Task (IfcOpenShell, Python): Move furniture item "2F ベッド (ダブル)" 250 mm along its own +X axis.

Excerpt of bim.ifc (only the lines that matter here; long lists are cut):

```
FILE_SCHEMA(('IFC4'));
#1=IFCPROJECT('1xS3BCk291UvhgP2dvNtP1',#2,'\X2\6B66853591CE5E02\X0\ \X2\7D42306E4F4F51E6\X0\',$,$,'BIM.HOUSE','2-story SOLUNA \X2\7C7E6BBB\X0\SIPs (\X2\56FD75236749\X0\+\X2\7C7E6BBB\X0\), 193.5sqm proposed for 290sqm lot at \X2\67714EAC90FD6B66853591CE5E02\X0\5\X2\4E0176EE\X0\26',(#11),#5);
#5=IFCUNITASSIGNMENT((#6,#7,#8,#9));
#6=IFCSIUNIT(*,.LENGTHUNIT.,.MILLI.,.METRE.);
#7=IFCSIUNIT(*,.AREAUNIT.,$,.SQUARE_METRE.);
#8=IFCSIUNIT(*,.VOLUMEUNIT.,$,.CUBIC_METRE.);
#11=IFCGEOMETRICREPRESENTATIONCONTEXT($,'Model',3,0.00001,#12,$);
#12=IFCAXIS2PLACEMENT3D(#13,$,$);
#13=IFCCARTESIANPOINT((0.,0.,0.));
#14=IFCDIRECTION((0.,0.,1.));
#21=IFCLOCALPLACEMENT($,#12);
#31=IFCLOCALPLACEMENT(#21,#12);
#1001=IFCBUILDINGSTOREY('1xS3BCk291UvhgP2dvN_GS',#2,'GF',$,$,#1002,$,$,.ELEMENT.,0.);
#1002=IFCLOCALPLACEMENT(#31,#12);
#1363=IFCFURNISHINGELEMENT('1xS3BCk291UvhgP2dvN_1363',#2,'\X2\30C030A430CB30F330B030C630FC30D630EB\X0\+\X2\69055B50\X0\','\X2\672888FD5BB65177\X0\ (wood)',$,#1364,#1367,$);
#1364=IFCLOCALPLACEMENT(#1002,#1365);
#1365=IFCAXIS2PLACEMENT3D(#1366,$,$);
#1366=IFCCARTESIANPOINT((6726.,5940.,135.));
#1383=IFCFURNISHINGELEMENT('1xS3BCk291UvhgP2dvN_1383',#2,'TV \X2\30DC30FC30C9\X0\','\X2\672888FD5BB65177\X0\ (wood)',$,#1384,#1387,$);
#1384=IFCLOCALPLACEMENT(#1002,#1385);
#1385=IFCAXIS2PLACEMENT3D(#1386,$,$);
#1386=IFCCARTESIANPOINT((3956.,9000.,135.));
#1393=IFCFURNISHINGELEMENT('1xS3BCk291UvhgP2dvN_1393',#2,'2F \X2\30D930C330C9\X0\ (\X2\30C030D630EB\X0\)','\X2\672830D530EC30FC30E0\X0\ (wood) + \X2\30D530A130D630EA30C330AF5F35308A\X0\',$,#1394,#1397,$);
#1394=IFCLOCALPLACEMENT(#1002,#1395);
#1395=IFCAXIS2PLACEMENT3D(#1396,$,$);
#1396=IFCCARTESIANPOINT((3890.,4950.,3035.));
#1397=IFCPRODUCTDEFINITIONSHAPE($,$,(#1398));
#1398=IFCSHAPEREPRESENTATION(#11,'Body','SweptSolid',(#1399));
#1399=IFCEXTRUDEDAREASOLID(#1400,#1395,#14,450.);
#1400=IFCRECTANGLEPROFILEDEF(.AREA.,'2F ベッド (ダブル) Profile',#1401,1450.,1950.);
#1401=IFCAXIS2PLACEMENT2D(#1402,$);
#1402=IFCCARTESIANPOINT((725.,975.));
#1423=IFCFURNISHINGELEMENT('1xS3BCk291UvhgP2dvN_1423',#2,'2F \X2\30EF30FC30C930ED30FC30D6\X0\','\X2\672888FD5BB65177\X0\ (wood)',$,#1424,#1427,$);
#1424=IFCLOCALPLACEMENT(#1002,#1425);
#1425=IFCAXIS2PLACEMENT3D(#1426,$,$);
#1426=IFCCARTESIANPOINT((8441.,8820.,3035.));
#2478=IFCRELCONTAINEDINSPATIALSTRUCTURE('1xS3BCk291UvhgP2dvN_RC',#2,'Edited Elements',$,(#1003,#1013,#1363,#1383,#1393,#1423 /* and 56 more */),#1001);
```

```python
import ifcopenshell
import ifcopenshell.api.geometry
import ifcopenshell.util.placement
import ifcopenshell.util.unit

model = ifcopenshell.open("bim.ifc")
unit_scale = ifcopenshell.util.unit.calculate_unit_scale(model)

item = model.by_guid("1xS3BCk291UvhgP2dvN_1393")
matrix = ifcopenshell.util.placement.get_local_placement(item.ObjectPlacement)
matrix[:3, 3] += matrix[:3, 0] * 0.25 / unit_scale
ifcopenshell.api.geometry.edit_object_placement(model, product=item, matrix=matrix, is_si=False)

print(ifcopenshell.util.placement.get_local_placement(item.ObjectPlacement).round(3) + 0.0)

model.write("bim_edited.ifc")
```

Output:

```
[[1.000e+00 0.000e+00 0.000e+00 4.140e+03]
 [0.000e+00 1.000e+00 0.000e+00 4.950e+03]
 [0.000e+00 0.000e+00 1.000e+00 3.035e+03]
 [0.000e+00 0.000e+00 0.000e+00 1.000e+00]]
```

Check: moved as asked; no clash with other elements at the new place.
